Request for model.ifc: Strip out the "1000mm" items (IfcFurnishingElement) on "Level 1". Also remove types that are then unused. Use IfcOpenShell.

First a look at what the model holds.

```python
import ifcopenshell
import ifcopenshell.util.element

model = ifcopenshell.open("model.ifc")
print(model.schema)
storey = next(s for s in model.by_type("IfcBuildingStorey") if s.Name == "Level 1")
furniture = [e for e in ifcopenshell.util.element.get_decomposition(storey) if e.is_a("IfcFurnishingElement")]
seen = {}
for e in furniture:
    element_type = ifcopenshell.util.element.get_type(e)
    name = element_type.Name if element_type not in (None, e) else None
    seen[name] = seen.get(name, 0) + 1
for name, count in sorted(seen.items(), key=str):
    print(count, "x", name)
```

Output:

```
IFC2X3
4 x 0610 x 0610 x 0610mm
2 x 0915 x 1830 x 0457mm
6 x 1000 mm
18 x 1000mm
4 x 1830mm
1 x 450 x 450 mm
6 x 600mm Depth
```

```python
import ifcopenshell
import ifcopenshell.api.root
import ifcopenshell.util.element

model = ifcopenshell.open("model.ifc")

storey = next(s for s in model.by_type("IfcBuildingStorey") if s.Name == "Level 1")
furniture = [e for e in ifcopenshell.util.element.get_decomposition(storey) if e.is_a("IfcFurnishingElement")]
targets = [e for e in furniture if (t := ifcopenshell.util.element.get_type(e)) not in (None, e) and t.Name == "1000mm"]
types = {ifcopenshell.util.element.get_type(e) for e in targets} - {None, *targets}

for e in targets:
    ifcopenshell.api.root.remove_product(model, product=e)
print(len(targets), "removed")

unused = [t for t in types if not ifcopenshell.util.element.get_types(t)]
for t in unused:
    ifcopenshell.api.root.remove_product(model, product=t)
print(len(unused), "unused types removed")

model.write("model_v2.ifc")
```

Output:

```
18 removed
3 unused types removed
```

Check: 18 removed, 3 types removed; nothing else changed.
